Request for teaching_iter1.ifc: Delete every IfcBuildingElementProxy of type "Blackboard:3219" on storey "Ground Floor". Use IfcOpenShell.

First a look at what the model holds.

```python
import ifcopenshell
import ifcopenshell.util.element

model = ifcopenshell.open("teaching_iter1.ifc")
print(model.schema)
storey = next(s for s in model.by_type("IfcBuildingStorey") if s.Name == "Ground Floor")
proxies = [e for e in ifcopenshell.util.element.get_decomposition(storey) if e.is_a("IfcBuildingElementProxy")]
seen = {}
for e in proxies:
    element_type = ifcopenshell.util.element.get_type(e)
    name = element_type.Name if element_type not in (None, e) else None
    seen[name] = seen.get(name, 0) + 1
for name, count in sorted(seen.items(), key=str):
    print(count, "x", name)
```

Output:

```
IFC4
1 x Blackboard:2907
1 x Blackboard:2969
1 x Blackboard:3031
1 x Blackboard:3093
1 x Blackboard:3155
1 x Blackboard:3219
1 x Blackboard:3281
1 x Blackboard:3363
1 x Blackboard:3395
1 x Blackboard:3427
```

```python
import ifcopenshell
import ifcopenshell.api.root
import ifcopenshell.util.element

model = ifcopenshell.open("teaching_iter1.ifc")

storey = next(s for s in model.by_type("IfcBuildingStorey") if s.Name == "Ground Floor")
proxies = [e for e in ifcopenshell.util.element.get_decomposition(storey) if e.is_a("IfcBuildingElementProxy")]
targets = [e for e in proxies if (t := ifcopenshell.util.element.get_type(e)) not in (None, e) and t.Name == "Blackboard:3219"]

for e in targets:
    ifcopenshell.api.root.remove_product(model, product=e)
print(len(targets), "removed")

model.write("teaching_iter1-out.ifc")
```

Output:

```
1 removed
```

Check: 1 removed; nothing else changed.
